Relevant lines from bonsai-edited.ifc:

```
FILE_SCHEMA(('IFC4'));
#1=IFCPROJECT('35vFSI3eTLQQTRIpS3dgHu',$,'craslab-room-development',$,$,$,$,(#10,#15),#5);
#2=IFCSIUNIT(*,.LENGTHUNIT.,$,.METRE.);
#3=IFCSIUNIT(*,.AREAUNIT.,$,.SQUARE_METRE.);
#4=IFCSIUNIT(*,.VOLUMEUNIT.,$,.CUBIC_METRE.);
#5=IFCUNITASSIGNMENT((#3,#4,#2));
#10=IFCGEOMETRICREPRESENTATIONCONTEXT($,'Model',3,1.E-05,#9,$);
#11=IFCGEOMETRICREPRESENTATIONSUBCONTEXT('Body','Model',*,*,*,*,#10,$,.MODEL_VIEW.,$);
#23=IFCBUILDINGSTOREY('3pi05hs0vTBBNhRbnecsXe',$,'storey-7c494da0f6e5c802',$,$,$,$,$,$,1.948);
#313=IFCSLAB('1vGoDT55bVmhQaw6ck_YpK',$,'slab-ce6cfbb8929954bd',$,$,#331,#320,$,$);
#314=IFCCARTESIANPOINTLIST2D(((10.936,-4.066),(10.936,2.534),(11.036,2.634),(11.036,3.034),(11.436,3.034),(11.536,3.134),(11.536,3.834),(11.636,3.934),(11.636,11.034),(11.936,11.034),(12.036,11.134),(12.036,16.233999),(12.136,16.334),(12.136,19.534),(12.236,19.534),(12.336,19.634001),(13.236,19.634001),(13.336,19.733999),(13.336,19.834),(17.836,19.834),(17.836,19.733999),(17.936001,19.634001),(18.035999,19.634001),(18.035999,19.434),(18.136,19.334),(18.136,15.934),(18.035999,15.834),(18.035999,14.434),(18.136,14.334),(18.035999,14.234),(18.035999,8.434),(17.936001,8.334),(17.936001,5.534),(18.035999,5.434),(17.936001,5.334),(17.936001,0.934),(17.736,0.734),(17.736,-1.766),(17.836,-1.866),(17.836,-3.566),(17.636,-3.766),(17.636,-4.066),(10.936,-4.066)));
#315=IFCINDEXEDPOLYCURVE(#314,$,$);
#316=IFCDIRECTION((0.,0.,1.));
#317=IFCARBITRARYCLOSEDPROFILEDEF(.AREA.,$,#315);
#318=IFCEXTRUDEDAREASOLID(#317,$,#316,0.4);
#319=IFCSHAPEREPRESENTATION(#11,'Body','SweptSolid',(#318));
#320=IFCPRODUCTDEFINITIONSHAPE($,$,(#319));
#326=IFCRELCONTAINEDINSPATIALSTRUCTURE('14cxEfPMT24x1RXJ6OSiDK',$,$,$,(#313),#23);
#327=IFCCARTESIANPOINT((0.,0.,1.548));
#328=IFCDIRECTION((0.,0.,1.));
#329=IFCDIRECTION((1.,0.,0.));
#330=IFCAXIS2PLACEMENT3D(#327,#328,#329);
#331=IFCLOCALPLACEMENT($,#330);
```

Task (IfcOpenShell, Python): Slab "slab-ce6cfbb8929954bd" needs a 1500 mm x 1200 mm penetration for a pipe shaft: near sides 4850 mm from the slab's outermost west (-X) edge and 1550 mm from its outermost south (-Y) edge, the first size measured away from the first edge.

```python
import numpy as np
import ifcopenshell
import ifcopenshell.api.feature
import ifcopenshell.api.geometry
import ifcopenshell.api.root
import ifcopenshell.geom
import ifcopenshell.util.placement
import ifcopenshell.util.representation
import ifcopenshell.util.shape
import ifcopenshell.util.unit

model = ifcopenshell.open("bonsai-edited.ifc")
unit_scale = ifcopenshell.util.unit.calculate_unit_scale(model)
settings = ifcopenshell.geom.settings()


def volume(element):
    """Net volume in cubic metres, openings subtracted."""
    shape = ifcopenshell.geom.create_shape(settings, element)
    return ifcopenshell.util.shape.get_volume(shape.geometry)


slab = model.by_guid("1vGoDT55bVmhQaw6ck_YpK")
before = volume(slab)

# Extent in the slab's own axes, in metres. The edges named are its -X and -Y sides.
slab_shape = ifcopenshell.geom.create_shape(settings, slab)
vertices = ifcopenshell.util.shape.get_vertices(slab_shape.geometry)
x_min, y_min, bottom = vertices.min(axis=0)
top = vertices[:, 2].max()

opening = ifcopenshell.api.root.create_entity(model, ifc_class="IfcOpeningElement", name="Pipe shaft opening", predefined_type="OPENING")
context = ifcopenshell.util.representation.get_context(model, "Model", "Body", "MODEL_VIEW")
width, depth = 1.5, 1.2
outline = [(0.0, 0.0), (width, 0.0), (width, depth), (0.0, depth), (0.0, 0.0)]
# Overshoot both faces by 50 mm so the cut is clean.
shape = ifcopenshell.api.geometry.add_slab_representation(
    model, context=context, depth=top - bottom + 0.1, polyline=outline
)
ifcopenshell.api.geometry.assign_representation(model, product=opening, representation=shape)

matrix = ifcopenshell.util.placement.get_local_placement(slab.ObjectPlacement)
matrix[:, 3] = matrix @ np.append(np.array([x_min + 4.85, y_min + 1.55, bottom - 0.05]) / unit_scale, 1.0)
ifcopenshell.api.geometry.edit_object_placement(model, product=opening, matrix=matrix, is_si=False)
ifcopenshell.api.feature.add_feature(model, feature=opening, element=slab)

after = volume(slab)

print(f"slab volume {before:.3f} -> {after:.3f} m3")

model.write("bonsai-edited_rev.ifc")
```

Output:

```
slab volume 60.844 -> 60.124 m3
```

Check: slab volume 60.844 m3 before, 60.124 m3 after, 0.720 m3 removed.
